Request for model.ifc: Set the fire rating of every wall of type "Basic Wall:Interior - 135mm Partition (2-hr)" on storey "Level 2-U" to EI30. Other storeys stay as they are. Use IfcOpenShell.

First a look at what the model holds.

```python
import ifcopenshell
import ifcopenshell.util.element

model = ifcopenshell.open("model.ifc")
print(model.schema)
storey = next(s for s in model.by_type("IfcBuildingStorey") if s.Name == "Level 2-U")
walls = [e for e in ifcopenshell.util.element.get_decomposition(storey) if e.is_a("IfcWall")]
seen = {}
for e in walls:
    element_type = ifcopenshell.util.element.get_type(e)
    key = (element_type.Name if element_type != e and element_type else None, ifcopenshell.util.element.get_pset(e, "Pset_WallCommon", "FireRating"))
    seen[key] = seen.get(key, 0) + 1
for (name, value), count in sorted(seen.items(), key=str):
    print(count, "x", name, "|", value)
```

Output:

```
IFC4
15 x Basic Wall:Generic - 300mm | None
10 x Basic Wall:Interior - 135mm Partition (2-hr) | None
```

```python
import ifcopenshell
import ifcopenshell.api.pset
import ifcopenshell.util.element

model = ifcopenshell.open("model.ifc")

storey = next(s for s in model.by_type("IfcBuildingStorey") if s.Name == "Level 2-U")
walls = [e for e in ifcopenshell.util.element.get_decomposition(storey) if e.is_a("IfcWall")]

count = 0
for e in walls:
    element_type = ifcopenshell.util.element.get_type(e)
    if element_type in (None, e) or element_type.Name != "Basic Wall:Interior - 135mm Partition (2-hr)":
        continue
    # add_pset returns the element's existing set when there is one.
    pset = ifcopenshell.api.pset.add_pset(model, product=e, name="Pset_WallCommon")
    ifcopenshell.api.pset.edit_pset(model, pset=pset, properties={"FireRating": "EI30"})
    count += 1

print(count, "walls updated")

model.write("model_edited.ifc")
```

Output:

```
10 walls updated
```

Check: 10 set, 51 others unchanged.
